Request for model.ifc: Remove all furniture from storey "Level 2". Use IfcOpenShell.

First a look at what the model holds.

```python
import ifcopenshell
import ifcopenshell.util.element

model = ifcopenshell.open("model.ifc")
print(model.schema)
storey = next(s for s in model.by_type("IfcBuildingStorey") if s.Name == "Level 2")
furniture = [e for e in ifcopenshell.util.element.get_decomposition(storey) if e.is_a("IfcFurnishingElement")]
seen = {}
for e in furniture:
    element_type = ifcopenshell.util.element.get_type(e)
    name = element_type.Name if element_type not in (None, e) else None
    seen[name] = seen.get(name, 0) + 1
for name, count in sorted(seen.items(), key=str):
    print(count, "x", name)
```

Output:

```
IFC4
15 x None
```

```python
import ifcopenshell
import ifcopenshell.api.root
import ifcopenshell.util.element

model = ifcopenshell.open("model.ifc")

storey = next(s for s in model.by_type("IfcBuildingStorey") if s.Name == "Level 2")
furniture = [e for e in ifcopenshell.util.element.get_decomposition(storey) if e.is_a("IfcFurnishingElement")]

for e in furniture:
    ifcopenshell.api.root.remove_product(model, product=e)
print(len(furniture), "removed")

model.write("model_updated.ifc")
```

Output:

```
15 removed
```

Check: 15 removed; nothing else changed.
